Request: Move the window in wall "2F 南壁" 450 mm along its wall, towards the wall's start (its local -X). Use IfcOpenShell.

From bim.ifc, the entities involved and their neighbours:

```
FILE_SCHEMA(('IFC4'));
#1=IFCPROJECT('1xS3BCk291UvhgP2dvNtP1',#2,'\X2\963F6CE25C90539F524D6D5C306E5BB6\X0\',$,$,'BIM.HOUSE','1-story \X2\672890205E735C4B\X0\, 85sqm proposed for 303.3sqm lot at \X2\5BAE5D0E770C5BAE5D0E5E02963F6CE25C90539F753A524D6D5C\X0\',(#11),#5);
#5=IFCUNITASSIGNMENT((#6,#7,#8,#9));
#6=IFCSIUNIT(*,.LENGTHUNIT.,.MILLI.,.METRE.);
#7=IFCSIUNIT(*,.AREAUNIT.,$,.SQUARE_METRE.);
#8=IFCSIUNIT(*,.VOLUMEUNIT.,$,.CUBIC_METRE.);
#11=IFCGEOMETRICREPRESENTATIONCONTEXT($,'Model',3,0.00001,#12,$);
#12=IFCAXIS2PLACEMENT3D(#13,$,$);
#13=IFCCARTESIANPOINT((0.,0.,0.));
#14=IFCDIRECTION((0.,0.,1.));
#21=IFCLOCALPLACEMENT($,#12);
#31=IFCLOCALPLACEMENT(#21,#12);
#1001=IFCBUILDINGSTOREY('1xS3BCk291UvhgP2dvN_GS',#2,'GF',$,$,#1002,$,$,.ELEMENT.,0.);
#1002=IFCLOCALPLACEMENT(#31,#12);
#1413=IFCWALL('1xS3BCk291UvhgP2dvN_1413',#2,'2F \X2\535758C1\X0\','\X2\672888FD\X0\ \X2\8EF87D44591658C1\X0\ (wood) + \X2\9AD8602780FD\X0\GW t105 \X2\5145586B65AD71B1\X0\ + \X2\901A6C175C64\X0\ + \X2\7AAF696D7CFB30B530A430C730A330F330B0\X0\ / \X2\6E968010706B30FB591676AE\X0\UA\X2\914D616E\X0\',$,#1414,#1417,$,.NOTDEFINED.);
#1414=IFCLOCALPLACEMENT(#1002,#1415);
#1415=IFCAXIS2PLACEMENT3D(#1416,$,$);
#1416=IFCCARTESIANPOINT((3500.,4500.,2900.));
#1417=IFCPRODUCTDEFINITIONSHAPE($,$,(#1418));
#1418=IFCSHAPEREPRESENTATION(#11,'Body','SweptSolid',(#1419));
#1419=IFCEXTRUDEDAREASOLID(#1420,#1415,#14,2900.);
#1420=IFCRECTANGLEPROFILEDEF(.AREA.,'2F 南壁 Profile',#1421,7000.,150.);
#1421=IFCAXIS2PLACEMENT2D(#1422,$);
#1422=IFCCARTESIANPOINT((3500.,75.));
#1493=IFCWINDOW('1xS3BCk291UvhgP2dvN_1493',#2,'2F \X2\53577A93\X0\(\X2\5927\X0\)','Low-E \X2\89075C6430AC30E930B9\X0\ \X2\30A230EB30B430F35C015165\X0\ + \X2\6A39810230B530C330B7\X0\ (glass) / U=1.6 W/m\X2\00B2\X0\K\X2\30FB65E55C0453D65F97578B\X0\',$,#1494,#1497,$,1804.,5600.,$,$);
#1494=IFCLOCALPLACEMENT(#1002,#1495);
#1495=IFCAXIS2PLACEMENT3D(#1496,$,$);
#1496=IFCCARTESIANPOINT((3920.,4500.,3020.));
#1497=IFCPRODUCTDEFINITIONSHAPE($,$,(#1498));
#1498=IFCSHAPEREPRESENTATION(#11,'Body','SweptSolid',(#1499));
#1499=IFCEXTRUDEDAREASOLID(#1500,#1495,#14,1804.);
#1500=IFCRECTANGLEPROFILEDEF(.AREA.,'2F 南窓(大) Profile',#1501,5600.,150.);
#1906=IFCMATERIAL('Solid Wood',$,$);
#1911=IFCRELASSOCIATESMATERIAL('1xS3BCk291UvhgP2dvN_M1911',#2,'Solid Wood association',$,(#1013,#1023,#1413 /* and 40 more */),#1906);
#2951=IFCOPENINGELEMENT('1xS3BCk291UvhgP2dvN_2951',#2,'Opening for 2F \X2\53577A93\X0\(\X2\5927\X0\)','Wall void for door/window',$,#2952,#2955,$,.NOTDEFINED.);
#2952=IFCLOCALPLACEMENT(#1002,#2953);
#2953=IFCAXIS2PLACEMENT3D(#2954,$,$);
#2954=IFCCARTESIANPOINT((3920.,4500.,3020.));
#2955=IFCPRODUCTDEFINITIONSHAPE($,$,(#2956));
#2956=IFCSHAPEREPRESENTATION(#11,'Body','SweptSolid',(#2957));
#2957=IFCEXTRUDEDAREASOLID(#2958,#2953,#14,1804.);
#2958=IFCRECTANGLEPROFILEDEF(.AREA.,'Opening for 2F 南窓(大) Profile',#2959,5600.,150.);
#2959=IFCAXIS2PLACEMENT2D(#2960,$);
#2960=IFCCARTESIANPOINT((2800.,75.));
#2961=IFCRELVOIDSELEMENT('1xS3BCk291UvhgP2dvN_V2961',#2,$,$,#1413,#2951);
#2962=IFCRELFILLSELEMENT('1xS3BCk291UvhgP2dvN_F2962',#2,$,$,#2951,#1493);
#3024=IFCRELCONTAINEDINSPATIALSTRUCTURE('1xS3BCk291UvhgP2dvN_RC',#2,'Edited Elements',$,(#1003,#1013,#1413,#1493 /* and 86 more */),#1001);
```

```python
import ifcopenshell
import ifcopenshell.api.geometry
import ifcopenshell.util.placement

model = ifcopenshell.open("bim.ifc")

window = model.by_guid("1xS3BCk291UvhgP2dvN_1493")
opening = window.FillsVoids[0].RelatingOpeningElement
wall = opening.VoidsElements[0].RelatingBuildingElement

wall_matrix = ifcopenshell.util.placement.get_local_placement(wall.ObjectPlacement)
shift = wall_matrix[:3, 0] * -450.0
before = ifcopenshell.util.placement.get_local_placement(window.ObjectPlacement)[:3, 3].copy()

# The window is not placed relative to its opening, so move both.
for product in (opening, window):
    matrix = ifcopenshell.util.placement.get_local_placement(product.ObjectPlacement)
    matrix[:3, 3] += shift
    ifcopenshell.api.geometry.edit_object_placement(model, product=product, matrix=matrix, is_si=False)

after = ifcopenshell.util.placement.get_local_placement(window.ObjectPlacement)[:3, 3]
print("window moved by", (after - before).round(3) + 0.0)

model.write("bim_updated.ifc")
```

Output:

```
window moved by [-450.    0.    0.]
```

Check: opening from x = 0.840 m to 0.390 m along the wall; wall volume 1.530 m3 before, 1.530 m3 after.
